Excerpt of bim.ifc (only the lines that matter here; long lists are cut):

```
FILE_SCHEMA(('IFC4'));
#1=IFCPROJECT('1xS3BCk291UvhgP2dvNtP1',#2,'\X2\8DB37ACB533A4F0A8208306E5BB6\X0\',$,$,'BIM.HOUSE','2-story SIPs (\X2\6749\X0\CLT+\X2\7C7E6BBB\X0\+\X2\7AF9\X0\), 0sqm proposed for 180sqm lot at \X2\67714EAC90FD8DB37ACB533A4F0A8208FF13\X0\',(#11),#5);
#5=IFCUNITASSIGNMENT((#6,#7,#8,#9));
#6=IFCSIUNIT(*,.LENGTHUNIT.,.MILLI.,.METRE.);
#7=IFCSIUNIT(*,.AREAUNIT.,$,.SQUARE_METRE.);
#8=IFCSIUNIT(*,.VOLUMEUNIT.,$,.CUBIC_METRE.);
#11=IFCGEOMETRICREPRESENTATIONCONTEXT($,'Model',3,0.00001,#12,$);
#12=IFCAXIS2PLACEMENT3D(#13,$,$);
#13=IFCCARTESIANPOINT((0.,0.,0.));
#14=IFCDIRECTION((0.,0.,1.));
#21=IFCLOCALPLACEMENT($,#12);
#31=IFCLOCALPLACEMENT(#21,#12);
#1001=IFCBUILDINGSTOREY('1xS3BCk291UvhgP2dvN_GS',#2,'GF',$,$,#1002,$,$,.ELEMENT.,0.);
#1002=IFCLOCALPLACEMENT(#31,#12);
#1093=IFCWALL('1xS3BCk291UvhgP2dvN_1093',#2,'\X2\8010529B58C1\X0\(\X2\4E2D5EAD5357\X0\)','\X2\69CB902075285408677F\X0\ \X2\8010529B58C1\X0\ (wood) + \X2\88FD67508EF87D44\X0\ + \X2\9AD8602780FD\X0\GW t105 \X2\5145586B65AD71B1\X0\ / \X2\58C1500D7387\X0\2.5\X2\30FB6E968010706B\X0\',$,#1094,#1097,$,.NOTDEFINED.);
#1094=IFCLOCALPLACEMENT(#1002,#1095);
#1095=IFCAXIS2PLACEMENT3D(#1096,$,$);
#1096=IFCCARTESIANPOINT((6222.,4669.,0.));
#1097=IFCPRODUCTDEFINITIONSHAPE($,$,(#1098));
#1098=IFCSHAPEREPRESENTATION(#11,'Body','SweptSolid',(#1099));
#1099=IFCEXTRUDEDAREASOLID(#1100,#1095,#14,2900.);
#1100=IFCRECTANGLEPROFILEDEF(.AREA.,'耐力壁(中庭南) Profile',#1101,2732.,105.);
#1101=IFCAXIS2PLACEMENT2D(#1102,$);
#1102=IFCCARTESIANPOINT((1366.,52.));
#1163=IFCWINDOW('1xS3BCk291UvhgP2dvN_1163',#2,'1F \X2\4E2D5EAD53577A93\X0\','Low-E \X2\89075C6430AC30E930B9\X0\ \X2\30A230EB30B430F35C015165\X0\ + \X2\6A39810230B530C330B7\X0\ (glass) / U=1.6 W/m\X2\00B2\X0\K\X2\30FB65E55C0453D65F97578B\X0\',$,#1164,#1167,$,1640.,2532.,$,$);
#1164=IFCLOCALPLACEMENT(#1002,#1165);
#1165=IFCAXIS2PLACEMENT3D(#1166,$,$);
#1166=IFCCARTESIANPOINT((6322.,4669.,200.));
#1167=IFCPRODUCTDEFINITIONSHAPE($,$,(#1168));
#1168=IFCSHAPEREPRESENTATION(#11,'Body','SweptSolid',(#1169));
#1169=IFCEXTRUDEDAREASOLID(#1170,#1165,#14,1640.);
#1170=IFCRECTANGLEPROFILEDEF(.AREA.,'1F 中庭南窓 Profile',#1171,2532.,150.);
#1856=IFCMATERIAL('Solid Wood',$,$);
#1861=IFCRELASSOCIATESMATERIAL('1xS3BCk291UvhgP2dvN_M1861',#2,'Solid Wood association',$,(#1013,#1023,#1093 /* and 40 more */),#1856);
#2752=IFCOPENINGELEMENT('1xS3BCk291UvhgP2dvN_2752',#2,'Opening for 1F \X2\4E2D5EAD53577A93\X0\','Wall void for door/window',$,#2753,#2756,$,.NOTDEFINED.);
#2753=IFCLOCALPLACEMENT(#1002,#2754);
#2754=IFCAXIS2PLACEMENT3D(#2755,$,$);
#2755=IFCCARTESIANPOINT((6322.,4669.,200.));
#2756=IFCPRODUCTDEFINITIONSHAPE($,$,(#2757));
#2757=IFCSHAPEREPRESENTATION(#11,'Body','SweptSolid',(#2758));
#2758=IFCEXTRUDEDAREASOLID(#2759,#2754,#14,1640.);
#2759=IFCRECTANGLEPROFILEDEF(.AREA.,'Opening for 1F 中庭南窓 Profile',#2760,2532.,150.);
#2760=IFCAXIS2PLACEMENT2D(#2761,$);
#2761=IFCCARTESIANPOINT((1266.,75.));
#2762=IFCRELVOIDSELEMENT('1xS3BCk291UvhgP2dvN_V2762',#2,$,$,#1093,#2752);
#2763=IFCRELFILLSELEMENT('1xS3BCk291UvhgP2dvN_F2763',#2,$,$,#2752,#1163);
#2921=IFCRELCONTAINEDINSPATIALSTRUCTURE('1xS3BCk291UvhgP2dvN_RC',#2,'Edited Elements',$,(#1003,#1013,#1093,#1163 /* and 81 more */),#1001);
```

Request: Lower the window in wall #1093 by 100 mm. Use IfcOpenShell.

```python
import numpy as np
import ifcopenshell
import ifcopenshell.api.geometry
import ifcopenshell.util.placement
import ifcopenshell.util.unit

model = ifcopenshell.open("bim.ifc")
unit_scale = ifcopenshell.util.unit.calculate_unit_scale(model)

window = model.by_guid("1xS3BCk291UvhgP2dvN_1163")
opening = window.FillsVoids[0].RelatingOpeningElement
dz = -0.1 / unit_scale

shift = np.array([0.0, 0.0, dz])
# The window is not placed relative to its opening, so move both.
for product in (opening, window):
    matrix = ifcopenshell.util.placement.get_local_placement(product.ObjectPlacement)
    matrix[:3, 3] += shift
    ifcopenshell.api.geometry.edit_object_placement(model, product=product, matrix=matrix, is_si=False)

print(f"moved by {dz * unit_scale:+.3f} m")

model.write("bim_v2.ifc")
```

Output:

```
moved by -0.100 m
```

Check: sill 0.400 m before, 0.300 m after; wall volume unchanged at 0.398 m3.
